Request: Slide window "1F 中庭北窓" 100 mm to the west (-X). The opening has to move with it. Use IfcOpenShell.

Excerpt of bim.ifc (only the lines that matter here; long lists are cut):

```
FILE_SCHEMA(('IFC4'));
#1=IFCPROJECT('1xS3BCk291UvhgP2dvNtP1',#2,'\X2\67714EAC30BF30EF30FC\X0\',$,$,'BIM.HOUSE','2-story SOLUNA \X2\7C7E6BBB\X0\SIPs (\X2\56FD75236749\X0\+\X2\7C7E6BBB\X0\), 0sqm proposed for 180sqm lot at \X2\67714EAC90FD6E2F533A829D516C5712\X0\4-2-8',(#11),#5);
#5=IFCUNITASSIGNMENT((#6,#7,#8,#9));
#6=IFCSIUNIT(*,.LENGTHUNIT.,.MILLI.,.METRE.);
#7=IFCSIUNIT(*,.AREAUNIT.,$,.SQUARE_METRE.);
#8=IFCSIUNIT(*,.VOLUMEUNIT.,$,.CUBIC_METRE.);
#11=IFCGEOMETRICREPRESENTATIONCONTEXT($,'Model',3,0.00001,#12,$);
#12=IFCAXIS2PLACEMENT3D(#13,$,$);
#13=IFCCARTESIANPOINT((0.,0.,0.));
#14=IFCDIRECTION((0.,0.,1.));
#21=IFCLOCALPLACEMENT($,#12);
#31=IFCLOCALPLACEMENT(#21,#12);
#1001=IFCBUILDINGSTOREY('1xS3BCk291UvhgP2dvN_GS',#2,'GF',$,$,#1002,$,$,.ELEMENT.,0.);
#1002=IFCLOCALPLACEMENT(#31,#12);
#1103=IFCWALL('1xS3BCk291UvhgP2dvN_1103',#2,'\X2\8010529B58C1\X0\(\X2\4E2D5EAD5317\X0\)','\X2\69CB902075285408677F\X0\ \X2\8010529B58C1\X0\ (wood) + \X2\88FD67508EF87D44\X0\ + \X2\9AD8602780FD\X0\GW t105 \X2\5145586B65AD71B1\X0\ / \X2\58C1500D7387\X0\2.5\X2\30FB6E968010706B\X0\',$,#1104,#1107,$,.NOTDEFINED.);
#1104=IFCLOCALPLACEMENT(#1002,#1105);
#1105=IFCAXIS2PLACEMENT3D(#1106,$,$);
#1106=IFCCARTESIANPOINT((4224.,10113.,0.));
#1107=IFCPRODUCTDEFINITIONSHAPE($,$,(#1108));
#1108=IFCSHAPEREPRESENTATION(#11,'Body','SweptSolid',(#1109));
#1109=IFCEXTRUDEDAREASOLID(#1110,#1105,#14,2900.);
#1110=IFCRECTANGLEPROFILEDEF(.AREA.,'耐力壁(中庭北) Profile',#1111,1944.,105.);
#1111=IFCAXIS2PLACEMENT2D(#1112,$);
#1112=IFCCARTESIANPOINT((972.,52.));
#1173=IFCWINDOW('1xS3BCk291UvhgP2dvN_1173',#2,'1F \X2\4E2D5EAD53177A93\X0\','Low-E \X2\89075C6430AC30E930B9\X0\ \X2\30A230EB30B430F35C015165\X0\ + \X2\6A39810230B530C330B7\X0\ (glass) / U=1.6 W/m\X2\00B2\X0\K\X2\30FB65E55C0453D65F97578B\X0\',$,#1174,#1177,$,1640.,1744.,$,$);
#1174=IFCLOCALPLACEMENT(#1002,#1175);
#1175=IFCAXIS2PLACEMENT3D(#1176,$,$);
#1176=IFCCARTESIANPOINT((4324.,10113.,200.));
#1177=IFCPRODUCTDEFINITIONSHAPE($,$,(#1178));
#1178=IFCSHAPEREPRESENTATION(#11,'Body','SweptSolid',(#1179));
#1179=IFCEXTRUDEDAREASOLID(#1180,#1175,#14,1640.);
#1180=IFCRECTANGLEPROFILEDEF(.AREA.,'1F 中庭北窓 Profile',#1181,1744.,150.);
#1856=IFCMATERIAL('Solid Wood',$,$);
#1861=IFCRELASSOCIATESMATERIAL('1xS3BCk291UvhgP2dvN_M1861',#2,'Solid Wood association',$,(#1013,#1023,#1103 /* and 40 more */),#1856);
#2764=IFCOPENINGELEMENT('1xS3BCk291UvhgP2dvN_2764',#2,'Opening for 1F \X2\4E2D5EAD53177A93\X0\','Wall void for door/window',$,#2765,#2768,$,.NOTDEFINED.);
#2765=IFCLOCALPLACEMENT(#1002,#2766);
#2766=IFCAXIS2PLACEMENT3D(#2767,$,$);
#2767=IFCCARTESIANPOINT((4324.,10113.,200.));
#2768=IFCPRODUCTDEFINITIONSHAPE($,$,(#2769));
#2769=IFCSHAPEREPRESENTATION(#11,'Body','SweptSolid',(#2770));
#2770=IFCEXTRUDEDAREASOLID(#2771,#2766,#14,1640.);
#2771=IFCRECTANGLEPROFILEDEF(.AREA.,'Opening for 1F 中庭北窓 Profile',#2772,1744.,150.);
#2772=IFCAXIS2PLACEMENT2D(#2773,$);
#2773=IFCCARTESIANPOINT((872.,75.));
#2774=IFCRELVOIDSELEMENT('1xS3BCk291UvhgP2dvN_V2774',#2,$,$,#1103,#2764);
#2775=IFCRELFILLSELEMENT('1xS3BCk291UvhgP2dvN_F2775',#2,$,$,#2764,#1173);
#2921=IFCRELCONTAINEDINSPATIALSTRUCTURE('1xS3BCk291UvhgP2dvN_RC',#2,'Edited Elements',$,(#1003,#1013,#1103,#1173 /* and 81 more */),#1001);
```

```python
import ifcopenshell
import ifcopenshell.api.geometry
import ifcopenshell.util.placement
import ifcopenshell.util.unit

model = ifcopenshell.open("bim.ifc")
unit_scale = ifcopenshell.util.unit.calculate_unit_scale(model)

window = model.by_id(1173)
opening = window.FillsVoids[0].RelatingOpeningElement
wall = opening.VoidsElements[0].RelatingBuildingElement

wall_matrix = ifcopenshell.util.placement.get_local_placement(wall.ObjectPlacement)
shift = wall_matrix[:3, 0] * -0.1 / unit_scale
before = ifcopenshell.util.placement.get_local_placement(window.ObjectPlacement)[:3, 3].copy()

# The window is not placed relative to its opening, so move both.
for product in (opening, window):
    matrix = ifcopenshell.util.placement.get_local_placement(product.ObjectPlacement)
    matrix[:3, 3] += shift
    ifcopenshell.api.geometry.edit_object_placement(model, product=product, matrix=matrix, is_si=False)

after = ifcopenshell.util.placement.get_local_placement(window.ObjectPlacement)[:3, 3]
print("window moved by", (after - before).round(3) + 0.0)

model.write("bim_edited.ifc")
```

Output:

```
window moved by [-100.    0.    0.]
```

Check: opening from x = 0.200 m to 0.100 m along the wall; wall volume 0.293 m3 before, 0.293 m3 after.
